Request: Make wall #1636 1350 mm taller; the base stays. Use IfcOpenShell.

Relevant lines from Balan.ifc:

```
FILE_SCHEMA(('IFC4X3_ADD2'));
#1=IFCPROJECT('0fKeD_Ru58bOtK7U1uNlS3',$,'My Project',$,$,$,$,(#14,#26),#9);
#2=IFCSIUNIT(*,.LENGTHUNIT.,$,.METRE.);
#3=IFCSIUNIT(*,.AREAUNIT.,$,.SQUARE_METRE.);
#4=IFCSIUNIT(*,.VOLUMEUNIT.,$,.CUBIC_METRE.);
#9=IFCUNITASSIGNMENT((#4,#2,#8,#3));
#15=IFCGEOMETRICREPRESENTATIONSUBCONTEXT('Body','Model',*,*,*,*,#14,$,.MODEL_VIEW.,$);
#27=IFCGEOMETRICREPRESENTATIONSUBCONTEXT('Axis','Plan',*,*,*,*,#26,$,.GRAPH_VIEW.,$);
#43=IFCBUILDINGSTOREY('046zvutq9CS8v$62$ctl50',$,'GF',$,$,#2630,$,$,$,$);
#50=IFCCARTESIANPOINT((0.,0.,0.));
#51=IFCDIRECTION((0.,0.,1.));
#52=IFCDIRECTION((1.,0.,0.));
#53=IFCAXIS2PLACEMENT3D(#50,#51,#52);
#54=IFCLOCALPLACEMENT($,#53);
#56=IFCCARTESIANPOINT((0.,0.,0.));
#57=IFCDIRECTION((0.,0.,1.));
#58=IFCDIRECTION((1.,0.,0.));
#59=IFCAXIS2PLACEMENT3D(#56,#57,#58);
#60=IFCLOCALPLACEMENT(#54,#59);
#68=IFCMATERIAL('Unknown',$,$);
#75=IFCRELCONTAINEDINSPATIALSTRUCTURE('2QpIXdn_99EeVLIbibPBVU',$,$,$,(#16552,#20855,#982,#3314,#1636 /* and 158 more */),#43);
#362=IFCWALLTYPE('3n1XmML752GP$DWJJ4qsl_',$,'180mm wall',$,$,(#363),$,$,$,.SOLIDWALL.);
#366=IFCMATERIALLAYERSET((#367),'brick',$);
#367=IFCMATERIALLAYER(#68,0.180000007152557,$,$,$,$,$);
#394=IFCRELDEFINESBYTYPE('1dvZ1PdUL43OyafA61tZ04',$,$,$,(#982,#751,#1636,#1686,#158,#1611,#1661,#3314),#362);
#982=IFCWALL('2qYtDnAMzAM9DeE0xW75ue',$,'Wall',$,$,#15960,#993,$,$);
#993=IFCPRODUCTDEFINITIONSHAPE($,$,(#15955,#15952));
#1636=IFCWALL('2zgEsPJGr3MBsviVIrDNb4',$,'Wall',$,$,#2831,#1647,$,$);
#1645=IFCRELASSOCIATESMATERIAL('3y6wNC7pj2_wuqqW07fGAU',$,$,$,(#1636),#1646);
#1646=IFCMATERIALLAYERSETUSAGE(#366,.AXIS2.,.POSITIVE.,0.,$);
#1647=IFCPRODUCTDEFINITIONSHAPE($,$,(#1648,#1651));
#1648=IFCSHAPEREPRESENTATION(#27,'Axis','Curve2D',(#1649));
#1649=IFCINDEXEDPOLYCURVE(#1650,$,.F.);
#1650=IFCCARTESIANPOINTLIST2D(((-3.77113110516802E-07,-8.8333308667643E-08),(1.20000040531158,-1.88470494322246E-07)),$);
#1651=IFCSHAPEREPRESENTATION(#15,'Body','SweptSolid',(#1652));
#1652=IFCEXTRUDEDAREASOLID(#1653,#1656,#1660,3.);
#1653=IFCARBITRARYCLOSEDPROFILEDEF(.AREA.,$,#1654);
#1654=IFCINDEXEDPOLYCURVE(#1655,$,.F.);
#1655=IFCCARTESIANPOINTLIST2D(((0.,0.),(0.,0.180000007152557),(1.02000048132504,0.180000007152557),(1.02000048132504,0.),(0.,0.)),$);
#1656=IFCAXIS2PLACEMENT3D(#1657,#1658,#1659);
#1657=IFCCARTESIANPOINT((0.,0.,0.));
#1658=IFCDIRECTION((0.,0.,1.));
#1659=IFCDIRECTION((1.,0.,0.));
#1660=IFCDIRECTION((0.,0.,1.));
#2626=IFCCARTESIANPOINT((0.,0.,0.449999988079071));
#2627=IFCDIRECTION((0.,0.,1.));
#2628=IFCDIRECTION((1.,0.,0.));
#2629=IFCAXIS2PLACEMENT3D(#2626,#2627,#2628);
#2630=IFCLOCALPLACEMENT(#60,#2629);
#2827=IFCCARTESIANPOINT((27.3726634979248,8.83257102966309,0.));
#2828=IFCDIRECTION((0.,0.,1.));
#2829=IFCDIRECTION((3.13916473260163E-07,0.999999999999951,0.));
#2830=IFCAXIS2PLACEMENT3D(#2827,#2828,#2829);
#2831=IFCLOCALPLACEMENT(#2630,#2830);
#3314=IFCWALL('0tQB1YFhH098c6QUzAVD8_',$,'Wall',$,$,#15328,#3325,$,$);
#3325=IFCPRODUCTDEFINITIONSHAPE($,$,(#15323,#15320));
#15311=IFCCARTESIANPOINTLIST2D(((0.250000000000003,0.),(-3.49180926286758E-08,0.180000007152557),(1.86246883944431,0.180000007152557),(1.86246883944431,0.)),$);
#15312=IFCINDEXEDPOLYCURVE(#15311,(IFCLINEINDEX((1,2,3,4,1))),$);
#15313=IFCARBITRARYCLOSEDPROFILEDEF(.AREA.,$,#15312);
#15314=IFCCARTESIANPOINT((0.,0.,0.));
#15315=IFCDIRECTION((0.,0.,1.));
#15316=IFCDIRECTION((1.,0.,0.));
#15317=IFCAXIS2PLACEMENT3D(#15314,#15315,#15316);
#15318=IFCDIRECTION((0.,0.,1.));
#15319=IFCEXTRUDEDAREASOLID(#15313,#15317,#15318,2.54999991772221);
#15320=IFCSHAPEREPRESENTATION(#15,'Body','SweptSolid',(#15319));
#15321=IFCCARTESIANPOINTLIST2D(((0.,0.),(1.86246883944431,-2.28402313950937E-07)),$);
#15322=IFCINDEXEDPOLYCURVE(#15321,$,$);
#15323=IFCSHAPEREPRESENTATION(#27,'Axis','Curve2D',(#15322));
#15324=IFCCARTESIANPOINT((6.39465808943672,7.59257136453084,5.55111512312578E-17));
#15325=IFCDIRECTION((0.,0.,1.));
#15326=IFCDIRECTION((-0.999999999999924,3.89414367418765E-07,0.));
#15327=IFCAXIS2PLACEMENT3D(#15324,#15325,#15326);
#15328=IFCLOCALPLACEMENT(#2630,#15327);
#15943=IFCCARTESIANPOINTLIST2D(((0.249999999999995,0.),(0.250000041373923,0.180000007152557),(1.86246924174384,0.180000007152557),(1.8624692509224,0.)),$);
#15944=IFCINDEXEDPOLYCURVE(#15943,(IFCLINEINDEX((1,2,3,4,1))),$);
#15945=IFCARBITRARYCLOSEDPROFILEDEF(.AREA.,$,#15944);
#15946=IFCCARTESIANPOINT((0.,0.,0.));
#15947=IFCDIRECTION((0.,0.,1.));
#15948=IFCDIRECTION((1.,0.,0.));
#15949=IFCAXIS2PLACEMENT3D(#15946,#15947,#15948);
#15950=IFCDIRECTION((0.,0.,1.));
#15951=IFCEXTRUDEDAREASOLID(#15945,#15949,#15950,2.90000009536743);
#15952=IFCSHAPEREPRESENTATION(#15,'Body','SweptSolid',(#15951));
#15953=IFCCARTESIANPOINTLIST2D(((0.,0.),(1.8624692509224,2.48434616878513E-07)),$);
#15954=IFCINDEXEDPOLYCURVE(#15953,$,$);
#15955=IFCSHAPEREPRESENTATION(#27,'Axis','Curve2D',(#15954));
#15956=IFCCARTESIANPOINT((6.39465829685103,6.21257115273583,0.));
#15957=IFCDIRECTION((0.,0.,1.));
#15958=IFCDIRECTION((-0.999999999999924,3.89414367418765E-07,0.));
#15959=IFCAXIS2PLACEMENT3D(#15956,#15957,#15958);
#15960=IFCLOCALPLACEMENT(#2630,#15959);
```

```python
import ifcopenshell
import ifcopenshell.geom
import ifcopenshell.util.representation
import ifcopenshell.util.shape
import ifcopenshell.util.unit

model = ifcopenshell.open("Balan.ifc")
unit_scale = ifcopenshell.util.unit.calculate_unit_scale(model)
settings = ifcopenshell.geom.settings()


def volume(element):
    """Net volume in cubic metres, openings subtracted."""
    shape = ifcopenshell.geom.create_shape(settings, element)
    return ifcopenshell.util.shape.get_volume(shape.geometry)


wall = model.by_id(1636)
before = volume(wall)

body = ifcopenshell.util.representation.get_representation(wall, "Model", "Body")
solid = body.Items[0]
old_height = solid.Depth
solid.Depth += 1.35 / unit_scale
after = volume(wall)

print(f"height {old_height:g} -> {solid.Depth:g}, volume {before:.3f} -> {after:.3f} m3")

model.write("Balan_v2.ifc")
```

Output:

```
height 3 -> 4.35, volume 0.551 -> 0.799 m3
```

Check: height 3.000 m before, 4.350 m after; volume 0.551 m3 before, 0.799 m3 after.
